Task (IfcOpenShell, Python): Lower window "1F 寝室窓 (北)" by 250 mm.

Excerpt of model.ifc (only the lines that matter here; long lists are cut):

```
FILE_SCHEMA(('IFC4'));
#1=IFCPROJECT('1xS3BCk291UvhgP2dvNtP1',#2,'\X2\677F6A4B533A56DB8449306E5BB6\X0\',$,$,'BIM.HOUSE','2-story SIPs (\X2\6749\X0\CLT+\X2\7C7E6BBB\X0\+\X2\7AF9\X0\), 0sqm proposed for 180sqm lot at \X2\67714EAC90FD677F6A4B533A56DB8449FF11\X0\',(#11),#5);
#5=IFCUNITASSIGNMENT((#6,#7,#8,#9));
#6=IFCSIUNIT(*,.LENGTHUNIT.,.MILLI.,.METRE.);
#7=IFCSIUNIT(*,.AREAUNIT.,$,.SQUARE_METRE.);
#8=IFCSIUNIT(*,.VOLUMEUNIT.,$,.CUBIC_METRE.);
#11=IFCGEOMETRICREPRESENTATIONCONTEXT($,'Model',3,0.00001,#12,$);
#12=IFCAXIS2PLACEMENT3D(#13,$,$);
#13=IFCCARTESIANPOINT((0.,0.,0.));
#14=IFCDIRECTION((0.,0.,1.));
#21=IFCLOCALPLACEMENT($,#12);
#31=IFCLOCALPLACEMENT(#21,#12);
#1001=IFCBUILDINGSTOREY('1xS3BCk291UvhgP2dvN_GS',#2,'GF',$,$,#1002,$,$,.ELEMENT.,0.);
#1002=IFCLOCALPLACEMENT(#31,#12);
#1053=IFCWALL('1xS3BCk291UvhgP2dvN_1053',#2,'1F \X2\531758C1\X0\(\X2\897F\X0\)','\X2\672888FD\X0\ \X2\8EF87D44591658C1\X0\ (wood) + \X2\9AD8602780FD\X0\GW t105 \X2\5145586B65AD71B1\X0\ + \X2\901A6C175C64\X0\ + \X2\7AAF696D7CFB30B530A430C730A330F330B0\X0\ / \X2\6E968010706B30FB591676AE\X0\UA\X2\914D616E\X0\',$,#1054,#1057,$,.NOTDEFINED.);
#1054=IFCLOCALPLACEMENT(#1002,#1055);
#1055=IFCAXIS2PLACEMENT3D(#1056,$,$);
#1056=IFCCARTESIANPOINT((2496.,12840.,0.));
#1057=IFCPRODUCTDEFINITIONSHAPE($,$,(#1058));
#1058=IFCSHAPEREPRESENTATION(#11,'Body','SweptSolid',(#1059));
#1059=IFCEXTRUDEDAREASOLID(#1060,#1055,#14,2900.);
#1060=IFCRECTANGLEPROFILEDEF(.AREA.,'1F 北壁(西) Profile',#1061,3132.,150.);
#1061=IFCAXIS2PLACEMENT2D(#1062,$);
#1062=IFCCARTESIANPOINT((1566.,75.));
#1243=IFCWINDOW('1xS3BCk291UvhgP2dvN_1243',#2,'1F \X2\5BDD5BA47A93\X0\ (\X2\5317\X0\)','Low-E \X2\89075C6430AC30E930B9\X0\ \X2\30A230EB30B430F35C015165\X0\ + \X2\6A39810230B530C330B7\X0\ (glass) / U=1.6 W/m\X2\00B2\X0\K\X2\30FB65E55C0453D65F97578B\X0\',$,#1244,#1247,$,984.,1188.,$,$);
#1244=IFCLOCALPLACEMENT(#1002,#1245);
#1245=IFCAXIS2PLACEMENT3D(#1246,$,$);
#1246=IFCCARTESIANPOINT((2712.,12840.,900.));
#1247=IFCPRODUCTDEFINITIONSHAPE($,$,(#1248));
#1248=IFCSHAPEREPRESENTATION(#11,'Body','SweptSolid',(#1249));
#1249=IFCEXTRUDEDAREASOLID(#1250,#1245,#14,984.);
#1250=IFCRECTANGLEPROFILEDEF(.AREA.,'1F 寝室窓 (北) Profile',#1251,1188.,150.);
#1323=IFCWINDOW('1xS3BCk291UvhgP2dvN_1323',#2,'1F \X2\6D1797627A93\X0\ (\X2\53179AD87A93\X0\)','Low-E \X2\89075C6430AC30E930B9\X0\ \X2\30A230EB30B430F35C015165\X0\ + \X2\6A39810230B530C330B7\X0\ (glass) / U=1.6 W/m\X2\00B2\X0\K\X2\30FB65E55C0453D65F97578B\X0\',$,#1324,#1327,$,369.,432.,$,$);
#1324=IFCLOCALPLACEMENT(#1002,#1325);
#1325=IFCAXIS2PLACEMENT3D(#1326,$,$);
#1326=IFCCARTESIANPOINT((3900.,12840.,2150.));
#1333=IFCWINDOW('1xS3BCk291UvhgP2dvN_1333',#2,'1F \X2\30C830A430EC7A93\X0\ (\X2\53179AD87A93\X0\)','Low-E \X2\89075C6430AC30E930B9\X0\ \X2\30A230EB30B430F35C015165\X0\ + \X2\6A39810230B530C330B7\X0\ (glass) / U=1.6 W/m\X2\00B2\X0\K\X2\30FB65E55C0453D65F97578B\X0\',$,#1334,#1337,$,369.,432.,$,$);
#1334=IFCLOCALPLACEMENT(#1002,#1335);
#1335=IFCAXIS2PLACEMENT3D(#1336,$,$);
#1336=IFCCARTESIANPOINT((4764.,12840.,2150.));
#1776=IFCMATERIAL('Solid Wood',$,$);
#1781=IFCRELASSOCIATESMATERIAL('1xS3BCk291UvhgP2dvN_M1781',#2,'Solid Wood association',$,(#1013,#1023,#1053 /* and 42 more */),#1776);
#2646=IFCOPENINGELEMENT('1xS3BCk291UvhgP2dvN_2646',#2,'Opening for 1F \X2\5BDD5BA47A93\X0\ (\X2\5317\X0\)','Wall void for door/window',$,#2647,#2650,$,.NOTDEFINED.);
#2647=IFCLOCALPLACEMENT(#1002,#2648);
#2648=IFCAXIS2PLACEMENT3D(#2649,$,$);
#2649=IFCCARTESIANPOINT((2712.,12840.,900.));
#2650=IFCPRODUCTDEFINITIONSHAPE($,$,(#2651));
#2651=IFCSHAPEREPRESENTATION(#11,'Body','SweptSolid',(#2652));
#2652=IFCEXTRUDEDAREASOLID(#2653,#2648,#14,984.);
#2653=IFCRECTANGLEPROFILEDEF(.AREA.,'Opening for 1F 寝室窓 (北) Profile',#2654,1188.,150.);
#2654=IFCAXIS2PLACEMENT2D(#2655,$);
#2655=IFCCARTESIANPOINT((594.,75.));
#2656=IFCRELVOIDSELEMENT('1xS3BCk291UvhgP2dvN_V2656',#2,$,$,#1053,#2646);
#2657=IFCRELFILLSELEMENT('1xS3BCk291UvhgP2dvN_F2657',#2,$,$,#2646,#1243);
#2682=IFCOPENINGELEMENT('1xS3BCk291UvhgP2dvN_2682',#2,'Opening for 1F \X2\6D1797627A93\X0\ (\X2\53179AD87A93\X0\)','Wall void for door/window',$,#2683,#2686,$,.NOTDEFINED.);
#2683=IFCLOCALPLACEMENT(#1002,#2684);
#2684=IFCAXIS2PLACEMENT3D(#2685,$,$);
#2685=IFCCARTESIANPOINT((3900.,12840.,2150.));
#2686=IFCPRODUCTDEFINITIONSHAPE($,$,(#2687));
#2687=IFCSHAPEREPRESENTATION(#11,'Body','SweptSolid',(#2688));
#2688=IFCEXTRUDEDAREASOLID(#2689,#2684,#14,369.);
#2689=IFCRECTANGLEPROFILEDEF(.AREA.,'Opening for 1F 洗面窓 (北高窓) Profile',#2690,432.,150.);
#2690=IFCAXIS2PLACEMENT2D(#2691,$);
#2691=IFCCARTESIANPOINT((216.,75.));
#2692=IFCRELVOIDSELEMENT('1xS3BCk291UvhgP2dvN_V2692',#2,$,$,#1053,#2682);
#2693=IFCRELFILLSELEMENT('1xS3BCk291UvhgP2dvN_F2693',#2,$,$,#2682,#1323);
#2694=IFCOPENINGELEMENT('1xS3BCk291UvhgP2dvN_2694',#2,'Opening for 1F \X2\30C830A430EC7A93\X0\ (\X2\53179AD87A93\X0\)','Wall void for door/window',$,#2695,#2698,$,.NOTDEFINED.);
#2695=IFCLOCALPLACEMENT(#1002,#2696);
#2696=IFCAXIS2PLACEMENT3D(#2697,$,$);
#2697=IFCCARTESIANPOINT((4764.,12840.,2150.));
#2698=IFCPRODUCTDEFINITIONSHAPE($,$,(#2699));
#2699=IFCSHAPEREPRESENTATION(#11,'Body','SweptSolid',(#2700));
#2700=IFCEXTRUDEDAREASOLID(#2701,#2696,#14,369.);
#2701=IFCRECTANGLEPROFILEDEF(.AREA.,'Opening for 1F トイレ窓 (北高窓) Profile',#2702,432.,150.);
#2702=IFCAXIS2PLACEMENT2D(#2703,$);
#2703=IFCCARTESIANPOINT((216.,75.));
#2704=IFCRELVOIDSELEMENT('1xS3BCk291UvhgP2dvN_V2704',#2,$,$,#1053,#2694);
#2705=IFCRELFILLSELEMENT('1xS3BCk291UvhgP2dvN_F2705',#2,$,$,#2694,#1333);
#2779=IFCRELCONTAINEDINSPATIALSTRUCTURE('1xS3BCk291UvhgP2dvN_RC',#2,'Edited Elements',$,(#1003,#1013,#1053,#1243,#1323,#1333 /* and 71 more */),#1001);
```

```python
import numpy as np
import ifcopenshell
import ifcopenshell.api.geometry
import ifcopenshell.util.placement
import ifcopenshell.util.unit

model = ifcopenshell.open("model.ifc")
unit_scale = ifcopenshell.util.unit.calculate_unit_scale(model)

window = model.by_guid("1xS3BCk291UvhgP2dvN_1243")
opening = window.FillsVoids[0].RelatingOpeningElement
dz = -250.0

shift = np.array([0.0, 0.0, dz])
# The window is not placed relative to its opening, so move both.
for product in (opening, window):
    matrix = ifcopenshell.util.placement.get_local_placement(product.ObjectPlacement)
    matrix[:3, 3] += shift
    ifcopenshell.api.geometry.edit_object_placement(model, product=product, matrix=matrix, is_si=False)

print(f"moved by {dz * unit_scale:+.3f} m")

model.write("model_v2.ifc")
```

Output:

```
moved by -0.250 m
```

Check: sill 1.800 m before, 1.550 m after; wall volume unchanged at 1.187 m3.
